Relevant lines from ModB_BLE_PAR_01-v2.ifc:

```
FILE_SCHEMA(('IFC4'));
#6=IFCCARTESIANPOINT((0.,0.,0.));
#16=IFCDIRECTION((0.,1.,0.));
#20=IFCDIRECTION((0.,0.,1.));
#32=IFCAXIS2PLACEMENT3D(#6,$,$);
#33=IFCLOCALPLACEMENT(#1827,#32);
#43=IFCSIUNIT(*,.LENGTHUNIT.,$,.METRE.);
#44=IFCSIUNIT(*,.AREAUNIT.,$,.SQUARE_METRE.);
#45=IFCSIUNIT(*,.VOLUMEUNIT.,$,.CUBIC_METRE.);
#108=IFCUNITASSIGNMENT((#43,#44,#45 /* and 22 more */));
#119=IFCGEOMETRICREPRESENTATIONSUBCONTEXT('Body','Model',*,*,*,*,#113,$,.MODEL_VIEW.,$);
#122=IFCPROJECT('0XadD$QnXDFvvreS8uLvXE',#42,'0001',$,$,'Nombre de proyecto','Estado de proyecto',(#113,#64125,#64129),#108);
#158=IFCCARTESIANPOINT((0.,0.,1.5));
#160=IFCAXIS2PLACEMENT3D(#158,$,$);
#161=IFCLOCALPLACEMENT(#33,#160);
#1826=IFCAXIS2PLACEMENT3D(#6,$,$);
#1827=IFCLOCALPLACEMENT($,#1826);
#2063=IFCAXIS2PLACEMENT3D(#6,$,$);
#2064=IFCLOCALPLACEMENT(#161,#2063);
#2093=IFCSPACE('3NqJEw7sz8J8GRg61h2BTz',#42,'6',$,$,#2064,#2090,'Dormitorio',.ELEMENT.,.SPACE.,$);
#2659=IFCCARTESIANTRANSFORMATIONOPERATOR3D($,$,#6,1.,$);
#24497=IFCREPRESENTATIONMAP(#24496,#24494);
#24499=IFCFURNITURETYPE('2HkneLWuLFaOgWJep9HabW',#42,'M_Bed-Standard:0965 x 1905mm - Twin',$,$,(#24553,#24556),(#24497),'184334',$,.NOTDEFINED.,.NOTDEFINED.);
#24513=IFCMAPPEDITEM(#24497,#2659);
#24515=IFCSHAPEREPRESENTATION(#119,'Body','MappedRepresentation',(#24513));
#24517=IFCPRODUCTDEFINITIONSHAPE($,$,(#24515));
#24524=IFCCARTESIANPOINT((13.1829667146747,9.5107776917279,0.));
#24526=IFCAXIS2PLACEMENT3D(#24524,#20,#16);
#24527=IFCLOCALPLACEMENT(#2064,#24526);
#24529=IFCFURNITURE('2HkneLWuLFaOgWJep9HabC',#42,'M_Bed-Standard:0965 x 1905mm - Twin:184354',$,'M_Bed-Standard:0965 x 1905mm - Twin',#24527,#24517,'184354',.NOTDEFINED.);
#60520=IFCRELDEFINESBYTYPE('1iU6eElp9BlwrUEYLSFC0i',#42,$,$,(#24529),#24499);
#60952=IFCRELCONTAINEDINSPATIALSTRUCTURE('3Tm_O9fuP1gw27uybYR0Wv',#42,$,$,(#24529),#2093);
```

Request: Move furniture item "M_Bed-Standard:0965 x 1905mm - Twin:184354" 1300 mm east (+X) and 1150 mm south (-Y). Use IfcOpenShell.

```python
import ifcopenshell
import ifcopenshell.api.geometry
import ifcopenshell.util.placement
import ifcopenshell.util.unit

model = ifcopenshell.open("ModB_BLE_PAR_01-v2.ifc")
unit_scale = ifcopenshell.util.unit.calculate_unit_scale(model)

item = model.by_guid("2HkneLWuLFaOgWJep9HabC")
matrix = ifcopenshell.util.placement.get_local_placement(item.ObjectPlacement)
matrix[0, 3] += 1.3 / unit_scale
matrix[1, 3] -= 1.15 / unit_scale
ifcopenshell.api.geometry.edit_object_placement(model, product=item, matrix=matrix, is_si=False)

print(ifcopenshell.util.placement.get_local_placement(item.ObjectPlacement).round(3) + 0.0)

model.write("ModB_BLE_PAR_01-v2_rev.ifc")
```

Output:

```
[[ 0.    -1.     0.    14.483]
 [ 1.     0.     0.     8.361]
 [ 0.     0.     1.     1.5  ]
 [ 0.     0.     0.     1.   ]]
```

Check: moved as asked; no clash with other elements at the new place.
